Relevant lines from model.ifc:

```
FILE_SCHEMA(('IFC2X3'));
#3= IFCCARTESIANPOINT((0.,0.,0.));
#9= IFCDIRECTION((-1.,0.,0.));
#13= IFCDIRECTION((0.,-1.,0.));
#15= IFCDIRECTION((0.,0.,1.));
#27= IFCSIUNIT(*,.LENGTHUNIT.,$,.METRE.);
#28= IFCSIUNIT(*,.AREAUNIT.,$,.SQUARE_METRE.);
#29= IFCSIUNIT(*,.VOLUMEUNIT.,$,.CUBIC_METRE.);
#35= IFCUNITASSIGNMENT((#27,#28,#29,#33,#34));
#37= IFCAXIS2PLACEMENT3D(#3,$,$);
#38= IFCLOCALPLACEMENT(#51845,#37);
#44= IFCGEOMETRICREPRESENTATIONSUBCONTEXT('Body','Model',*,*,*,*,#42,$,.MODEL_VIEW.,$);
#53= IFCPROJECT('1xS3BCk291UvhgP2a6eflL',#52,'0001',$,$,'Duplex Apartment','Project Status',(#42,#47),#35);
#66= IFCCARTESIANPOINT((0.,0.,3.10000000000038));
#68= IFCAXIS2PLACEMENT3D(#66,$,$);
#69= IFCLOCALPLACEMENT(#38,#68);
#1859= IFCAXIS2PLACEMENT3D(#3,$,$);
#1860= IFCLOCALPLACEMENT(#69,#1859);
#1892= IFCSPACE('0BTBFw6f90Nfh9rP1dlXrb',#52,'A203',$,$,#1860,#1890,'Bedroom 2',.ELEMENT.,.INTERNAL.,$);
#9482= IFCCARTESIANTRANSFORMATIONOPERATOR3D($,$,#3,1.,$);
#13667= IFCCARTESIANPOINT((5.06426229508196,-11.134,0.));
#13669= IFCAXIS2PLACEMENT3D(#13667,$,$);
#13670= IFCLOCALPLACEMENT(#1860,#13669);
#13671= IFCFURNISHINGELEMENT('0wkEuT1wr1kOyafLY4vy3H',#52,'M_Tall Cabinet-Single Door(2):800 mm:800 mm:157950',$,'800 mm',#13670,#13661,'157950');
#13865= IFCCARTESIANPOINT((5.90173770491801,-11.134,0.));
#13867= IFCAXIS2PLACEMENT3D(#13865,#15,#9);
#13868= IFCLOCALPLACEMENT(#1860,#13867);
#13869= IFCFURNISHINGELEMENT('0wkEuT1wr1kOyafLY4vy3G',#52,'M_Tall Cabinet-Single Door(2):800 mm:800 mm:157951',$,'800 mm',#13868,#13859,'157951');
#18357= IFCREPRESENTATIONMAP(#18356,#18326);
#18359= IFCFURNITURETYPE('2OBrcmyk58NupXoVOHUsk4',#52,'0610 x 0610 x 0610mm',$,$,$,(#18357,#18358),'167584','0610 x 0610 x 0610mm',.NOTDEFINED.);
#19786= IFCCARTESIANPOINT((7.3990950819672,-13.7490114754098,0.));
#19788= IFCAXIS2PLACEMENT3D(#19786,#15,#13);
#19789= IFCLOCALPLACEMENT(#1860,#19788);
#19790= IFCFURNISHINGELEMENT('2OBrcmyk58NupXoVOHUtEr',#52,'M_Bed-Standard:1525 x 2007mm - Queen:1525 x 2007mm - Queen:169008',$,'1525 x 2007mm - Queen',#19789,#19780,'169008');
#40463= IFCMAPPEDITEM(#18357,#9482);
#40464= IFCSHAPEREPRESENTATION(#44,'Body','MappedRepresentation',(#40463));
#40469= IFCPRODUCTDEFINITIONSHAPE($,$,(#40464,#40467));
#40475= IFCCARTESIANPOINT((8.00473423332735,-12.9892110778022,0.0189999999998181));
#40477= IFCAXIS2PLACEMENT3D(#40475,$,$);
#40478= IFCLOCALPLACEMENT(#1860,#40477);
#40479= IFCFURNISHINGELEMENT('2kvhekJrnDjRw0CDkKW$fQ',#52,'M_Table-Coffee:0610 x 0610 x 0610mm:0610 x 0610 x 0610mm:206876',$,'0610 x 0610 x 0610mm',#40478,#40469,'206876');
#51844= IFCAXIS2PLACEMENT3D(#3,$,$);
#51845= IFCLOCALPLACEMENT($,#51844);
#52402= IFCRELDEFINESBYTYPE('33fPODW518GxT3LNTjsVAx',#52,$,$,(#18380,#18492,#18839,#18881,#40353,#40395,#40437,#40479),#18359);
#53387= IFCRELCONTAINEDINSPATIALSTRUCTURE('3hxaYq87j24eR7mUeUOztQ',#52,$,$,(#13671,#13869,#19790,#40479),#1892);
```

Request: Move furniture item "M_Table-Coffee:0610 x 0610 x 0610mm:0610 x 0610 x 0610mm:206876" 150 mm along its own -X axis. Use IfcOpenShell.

```python
import ifcopenshell
import ifcopenshell.api.geometry
import ifcopenshell.util.placement

model = ifcopenshell.open("model.ifc")

item = model.by_id(40479)
matrix = ifcopenshell.util.placement.get_local_placement(item.ObjectPlacement)
matrix[:3, 3] -= matrix[:3, 0] * 0.15
ifcopenshell.api.geometry.edit_object_placement(model, product=item, matrix=matrix, is_si=False)

print(ifcopenshell.util.placement.get_local_placement(item.ObjectPlacement).round(3) + 0.0)

model.write("model_v2.ifc")
```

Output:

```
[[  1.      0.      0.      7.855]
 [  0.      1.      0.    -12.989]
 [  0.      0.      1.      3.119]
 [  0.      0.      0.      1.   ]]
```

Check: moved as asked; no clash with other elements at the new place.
